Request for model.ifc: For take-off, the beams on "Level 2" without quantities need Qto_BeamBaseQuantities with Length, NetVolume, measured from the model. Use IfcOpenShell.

First a look at what the model holds.

```python
import ifcopenshell
import ifcopenshell.util.element
import ifcopenshell.util.unit

model = ifcopenshell.open("model.ifc")
print(model.schema)
for unit_type in ("LENGTHUNIT", "AREAUNIT", "VOLUMEUNIT"):
    print(unit_type, ifcopenshell.util.unit.calculate_unit_scale(model, unit_type))
storey = next(s for s in model.by_type("IfcBuildingStorey") if s.Name == "Level 2")
beams = [e for e in ifcopenshell.util.element.get_decomposition(storey) if e.is_a("IfcBeam")]
for e in sorted(beams, key=lambda e: e.id()):
    print(e.id(), e.is_a(), e.Name, list(ifcopenshell.util.element.get_psets(e, qtos_only=True)), sep=" | ")
```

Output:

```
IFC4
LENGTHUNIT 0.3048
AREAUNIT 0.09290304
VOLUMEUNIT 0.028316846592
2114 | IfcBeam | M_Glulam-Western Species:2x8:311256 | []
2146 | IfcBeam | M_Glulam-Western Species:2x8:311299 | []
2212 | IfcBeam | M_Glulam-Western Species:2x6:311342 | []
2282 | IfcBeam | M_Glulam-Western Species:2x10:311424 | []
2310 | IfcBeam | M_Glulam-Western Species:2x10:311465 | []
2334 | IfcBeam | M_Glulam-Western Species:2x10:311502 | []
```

```python
import ifcopenshell
import ifcopenshell.api.pset
import ifcopenshell.geom
import ifcopenshell.util.element
import ifcopenshell.util.shape
import ifcopenshell.util.unit

model = ifcopenshell.open("model.ifc")
unit_scale = ifcopenshell.util.unit.calculate_unit_scale(model)
volume_scale = ifcopenshell.util.unit.calculate_unit_scale(model, "VOLUMEUNIT")
settings = ifcopenshell.geom.settings()

storey = next(s for s in model.by_type("IfcBuildingStorey") if s.Name == "Level 2")
beams = [e for e in ifcopenshell.util.element.get_decomposition(storey) if e.is_a("IfcBeam")]

for e in sorted(beams, key=lambda e: e.id()):
    if ifcopenshell.util.element.get_psets(e, qtos_only=True, should_inherit=False):
        continue
    # Geometry comes back in metres, in the element's own axes.
    shape = ifcopenshell.geom.create_shape(settings, e)
    values = {
        "Length": ifcopenshell.util.shape.get_max_xyz(shape.geometry) / unit_scale,
        "NetVolume": ifcopenshell.util.shape.get_volume(shape.geometry) / volume_scale,
    }
    qto = ifcopenshell.api.pset.add_qto(model, product=e, name="Qto_BeamBaseQuantities")
    ifcopenshell.api.pset.edit_qto(model, qto=qto, properties=values)
    print(e.id(), {k: round(v, 3) for k, v in values.items()})

model.write("model_rev.ifc")
```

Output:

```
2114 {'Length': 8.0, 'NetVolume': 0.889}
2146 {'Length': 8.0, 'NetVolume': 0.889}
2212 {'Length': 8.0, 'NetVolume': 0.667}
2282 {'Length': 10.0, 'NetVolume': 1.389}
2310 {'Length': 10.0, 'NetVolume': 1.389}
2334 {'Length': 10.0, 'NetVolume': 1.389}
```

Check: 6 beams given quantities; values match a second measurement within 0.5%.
